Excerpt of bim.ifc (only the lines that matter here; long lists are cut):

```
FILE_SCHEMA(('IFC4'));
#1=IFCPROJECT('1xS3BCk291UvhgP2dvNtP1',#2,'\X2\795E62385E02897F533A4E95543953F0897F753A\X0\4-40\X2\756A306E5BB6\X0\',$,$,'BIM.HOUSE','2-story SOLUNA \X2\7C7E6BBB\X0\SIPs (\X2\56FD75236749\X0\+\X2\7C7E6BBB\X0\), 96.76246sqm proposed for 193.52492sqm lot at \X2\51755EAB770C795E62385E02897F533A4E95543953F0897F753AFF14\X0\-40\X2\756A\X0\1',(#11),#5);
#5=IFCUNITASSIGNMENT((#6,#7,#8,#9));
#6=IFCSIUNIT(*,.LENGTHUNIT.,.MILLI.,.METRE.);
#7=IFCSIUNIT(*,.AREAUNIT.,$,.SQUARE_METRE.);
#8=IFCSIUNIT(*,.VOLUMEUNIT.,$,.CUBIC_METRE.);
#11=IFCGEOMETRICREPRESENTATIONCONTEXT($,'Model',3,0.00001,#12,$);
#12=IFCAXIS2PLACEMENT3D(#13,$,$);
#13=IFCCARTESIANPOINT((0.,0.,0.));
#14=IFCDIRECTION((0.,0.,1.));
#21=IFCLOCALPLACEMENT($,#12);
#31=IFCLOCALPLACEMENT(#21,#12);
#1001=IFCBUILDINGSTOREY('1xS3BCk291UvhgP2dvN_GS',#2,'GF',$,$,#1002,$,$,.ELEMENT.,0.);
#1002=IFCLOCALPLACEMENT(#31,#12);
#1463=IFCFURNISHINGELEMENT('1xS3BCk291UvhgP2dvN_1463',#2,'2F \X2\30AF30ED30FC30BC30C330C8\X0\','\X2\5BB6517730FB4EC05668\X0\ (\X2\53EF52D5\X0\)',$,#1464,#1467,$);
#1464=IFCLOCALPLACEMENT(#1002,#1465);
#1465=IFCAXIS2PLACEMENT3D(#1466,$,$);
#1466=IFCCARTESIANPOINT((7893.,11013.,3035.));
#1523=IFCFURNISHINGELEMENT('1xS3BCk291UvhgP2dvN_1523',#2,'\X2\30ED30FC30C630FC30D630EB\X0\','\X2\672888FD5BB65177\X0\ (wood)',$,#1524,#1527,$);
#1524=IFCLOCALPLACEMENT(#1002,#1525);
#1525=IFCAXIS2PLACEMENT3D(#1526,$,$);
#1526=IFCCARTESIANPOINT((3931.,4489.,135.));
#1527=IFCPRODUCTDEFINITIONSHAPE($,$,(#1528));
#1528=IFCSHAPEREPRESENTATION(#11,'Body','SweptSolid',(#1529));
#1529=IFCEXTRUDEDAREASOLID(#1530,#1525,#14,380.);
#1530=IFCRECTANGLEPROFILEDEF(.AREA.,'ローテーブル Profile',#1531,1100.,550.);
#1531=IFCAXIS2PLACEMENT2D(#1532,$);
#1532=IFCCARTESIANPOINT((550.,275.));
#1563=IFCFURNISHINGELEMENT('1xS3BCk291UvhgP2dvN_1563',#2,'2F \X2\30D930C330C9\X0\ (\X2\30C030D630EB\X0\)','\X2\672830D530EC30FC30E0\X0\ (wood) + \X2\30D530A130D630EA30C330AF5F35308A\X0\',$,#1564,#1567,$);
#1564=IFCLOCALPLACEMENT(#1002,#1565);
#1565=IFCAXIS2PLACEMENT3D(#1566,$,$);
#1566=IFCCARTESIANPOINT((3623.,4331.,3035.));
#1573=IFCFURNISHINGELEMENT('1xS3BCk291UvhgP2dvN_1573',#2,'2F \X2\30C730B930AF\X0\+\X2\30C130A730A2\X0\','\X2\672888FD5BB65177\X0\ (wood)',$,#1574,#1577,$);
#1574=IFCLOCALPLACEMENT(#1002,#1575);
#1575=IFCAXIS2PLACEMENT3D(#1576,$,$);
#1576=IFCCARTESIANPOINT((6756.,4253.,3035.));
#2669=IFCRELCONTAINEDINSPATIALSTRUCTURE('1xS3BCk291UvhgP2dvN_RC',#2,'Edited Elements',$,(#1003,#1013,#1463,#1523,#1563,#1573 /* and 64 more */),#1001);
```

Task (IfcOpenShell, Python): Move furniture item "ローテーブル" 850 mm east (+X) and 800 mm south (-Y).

```python
import ifcopenshell
import ifcopenshell.api.geometry
import ifcopenshell.util.placement
import ifcopenshell.util.unit

model = ifcopenshell.open("bim.ifc")
unit_scale = ifcopenshell.util.unit.calculate_unit_scale(model)

item = model.by_id(1523)
matrix = ifcopenshell.util.placement.get_local_placement(item.ObjectPlacement)
matrix[0, 3] += 0.85 / unit_scale
matrix[1, 3] -= 0.8 / unit_scale
ifcopenshell.api.geometry.edit_object_placement(model, product=item, matrix=matrix, is_si=False)

print(ifcopenshell.util.placement.get_local_placement(item.ObjectPlacement).round(3) + 0.0)

model.write("bim-out.ifc")
```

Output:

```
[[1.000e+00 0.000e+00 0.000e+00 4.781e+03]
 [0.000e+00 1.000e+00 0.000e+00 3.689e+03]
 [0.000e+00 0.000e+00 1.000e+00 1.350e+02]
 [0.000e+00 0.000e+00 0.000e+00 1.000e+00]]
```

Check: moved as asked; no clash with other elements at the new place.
